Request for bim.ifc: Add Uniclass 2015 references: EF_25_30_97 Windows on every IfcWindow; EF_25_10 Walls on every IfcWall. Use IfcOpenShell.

First a look at what the model holds.

```python
import ifcopenshell

model = ifcopenshell.open("bim.ifc")
print(model.schema)
print("classifications:", [c.Name for c in model.by_type("IfcClassification")])
for ifc_class in ("IfcDoor", "IfcRoof", "IfcStair", "IfcWall", "IfcWindow"):
    print(ifc_class, len(model.by_type(ifc_class)))
```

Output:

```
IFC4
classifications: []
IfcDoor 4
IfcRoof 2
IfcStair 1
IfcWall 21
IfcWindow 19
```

```python
import ifcopenshell
import ifcopenshell.api.classification

model = ifcopenshell.open("bim.ifc")

system = ifcopenshell.api.classification.add_classification(model, classification="Uniclass 2015")

codes = {
    "IfcWindow": ("EF_25_30_97", "Windows"),
    "IfcWall": ("EF_25_10", "Walls"),
}
for ifc_class, (code, name) in codes.items():
    products = model.by_type(ifc_class)
    ifcopenshell.api.classification.add_reference(
        model, products=products, classification=system, identification=code, name=name
    )
    print(code, len(products))

model.write("bim_v2.ifc")
```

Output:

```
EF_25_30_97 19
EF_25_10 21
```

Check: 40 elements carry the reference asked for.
